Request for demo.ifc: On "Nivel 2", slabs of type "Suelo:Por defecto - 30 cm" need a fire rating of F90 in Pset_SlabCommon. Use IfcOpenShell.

First a look at what the model holds.

```python
import ifcopenshell
import ifcopenshell.util.element

model = ifcopenshell.open("demo.ifc")
print(model.schema)
storey = next(s for s in model.by_type("IfcBuildingStorey") if s.Name == "Nivel 2")
slabs = [e for e in ifcopenshell.util.element.get_decomposition(storey) if e.is_a("IfcSlab")]
seen = {}
for e in slabs:
    element_type = ifcopenshell.util.element.get_type(e)
    key = (element_type.Name if element_type != e and element_type else None, ifcopenshell.util.element.get_pset(e, "Pset_SlabCommon", "FireRating"))
    seen[key] = seen.get(key, 0) + 1
for (name, value), count in sorted(seen.items(), key=str):
    print(count, "x", name, "|", value)
```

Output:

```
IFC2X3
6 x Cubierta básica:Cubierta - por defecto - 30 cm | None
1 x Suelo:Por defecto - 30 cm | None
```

```python
import ifcopenshell
import ifcopenshell.api.pset
import ifcopenshell.util.element

model = ifcopenshell.open("demo.ifc")

storey = next(s for s in model.by_type("IfcBuildingStorey") if s.Name == "Nivel 2")
slabs = [e for e in ifcopenshell.util.element.get_decomposition(storey) if e.is_a("IfcSlab")]

count = 0
for e in slabs:
    element_type = ifcopenshell.util.element.get_type(e)
    if element_type in (None, e) or element_type.Name != "Suelo:Por defecto - 30 cm":
        continue
    # add_pset returns the element's existing set when there is one.
    pset = ifcopenshell.api.pset.add_pset(model, product=e, name="Pset_SlabCommon")
    ifcopenshell.api.pset.edit_pset(model, pset=pset, properties={"FireRating": "F90"})
    count += 1

print(count, "slabs updated")

model.write("demo_v2.ifc")
```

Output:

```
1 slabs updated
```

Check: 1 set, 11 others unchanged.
